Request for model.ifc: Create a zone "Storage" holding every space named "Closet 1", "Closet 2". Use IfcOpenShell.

First a look at what the model holds.

```python
import ifcopenshell

model = ifcopenshell.open("model.ifc")
print(model.schema)
seen = {}
for space in model.by_type("IfcSpace"):
    seen[space.LongName] = seen.get(space.LongName, 0) + 1
for name, count in sorted(seen.items(), key=str):
    print(count, "x", name)
print("zones:", [z.Name for z in model.by_type("IfcZone")][:20])
```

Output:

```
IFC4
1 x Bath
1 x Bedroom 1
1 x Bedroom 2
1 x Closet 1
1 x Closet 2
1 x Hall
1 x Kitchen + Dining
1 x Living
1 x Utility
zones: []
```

```python
import ifcopenshell
import ifcopenshell.api.group
import ifcopenshell.api.root

model = ifcopenshell.open("model.ifc")

names = {"Closet 1", "Closet 2"}
spaces = [s for s in model.by_type("IfcSpace") if s.LongName in names]

zone = ifcopenshell.api.root.create_entity(model, ifc_class="IfcZone", name="Storage")
ifcopenshell.api.group.assign_group(model, products=spaces, group=zone)
print(len(spaces), "spaces in", zone.Name)

model.write("model_updated.ifc")
```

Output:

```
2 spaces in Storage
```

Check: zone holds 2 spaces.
